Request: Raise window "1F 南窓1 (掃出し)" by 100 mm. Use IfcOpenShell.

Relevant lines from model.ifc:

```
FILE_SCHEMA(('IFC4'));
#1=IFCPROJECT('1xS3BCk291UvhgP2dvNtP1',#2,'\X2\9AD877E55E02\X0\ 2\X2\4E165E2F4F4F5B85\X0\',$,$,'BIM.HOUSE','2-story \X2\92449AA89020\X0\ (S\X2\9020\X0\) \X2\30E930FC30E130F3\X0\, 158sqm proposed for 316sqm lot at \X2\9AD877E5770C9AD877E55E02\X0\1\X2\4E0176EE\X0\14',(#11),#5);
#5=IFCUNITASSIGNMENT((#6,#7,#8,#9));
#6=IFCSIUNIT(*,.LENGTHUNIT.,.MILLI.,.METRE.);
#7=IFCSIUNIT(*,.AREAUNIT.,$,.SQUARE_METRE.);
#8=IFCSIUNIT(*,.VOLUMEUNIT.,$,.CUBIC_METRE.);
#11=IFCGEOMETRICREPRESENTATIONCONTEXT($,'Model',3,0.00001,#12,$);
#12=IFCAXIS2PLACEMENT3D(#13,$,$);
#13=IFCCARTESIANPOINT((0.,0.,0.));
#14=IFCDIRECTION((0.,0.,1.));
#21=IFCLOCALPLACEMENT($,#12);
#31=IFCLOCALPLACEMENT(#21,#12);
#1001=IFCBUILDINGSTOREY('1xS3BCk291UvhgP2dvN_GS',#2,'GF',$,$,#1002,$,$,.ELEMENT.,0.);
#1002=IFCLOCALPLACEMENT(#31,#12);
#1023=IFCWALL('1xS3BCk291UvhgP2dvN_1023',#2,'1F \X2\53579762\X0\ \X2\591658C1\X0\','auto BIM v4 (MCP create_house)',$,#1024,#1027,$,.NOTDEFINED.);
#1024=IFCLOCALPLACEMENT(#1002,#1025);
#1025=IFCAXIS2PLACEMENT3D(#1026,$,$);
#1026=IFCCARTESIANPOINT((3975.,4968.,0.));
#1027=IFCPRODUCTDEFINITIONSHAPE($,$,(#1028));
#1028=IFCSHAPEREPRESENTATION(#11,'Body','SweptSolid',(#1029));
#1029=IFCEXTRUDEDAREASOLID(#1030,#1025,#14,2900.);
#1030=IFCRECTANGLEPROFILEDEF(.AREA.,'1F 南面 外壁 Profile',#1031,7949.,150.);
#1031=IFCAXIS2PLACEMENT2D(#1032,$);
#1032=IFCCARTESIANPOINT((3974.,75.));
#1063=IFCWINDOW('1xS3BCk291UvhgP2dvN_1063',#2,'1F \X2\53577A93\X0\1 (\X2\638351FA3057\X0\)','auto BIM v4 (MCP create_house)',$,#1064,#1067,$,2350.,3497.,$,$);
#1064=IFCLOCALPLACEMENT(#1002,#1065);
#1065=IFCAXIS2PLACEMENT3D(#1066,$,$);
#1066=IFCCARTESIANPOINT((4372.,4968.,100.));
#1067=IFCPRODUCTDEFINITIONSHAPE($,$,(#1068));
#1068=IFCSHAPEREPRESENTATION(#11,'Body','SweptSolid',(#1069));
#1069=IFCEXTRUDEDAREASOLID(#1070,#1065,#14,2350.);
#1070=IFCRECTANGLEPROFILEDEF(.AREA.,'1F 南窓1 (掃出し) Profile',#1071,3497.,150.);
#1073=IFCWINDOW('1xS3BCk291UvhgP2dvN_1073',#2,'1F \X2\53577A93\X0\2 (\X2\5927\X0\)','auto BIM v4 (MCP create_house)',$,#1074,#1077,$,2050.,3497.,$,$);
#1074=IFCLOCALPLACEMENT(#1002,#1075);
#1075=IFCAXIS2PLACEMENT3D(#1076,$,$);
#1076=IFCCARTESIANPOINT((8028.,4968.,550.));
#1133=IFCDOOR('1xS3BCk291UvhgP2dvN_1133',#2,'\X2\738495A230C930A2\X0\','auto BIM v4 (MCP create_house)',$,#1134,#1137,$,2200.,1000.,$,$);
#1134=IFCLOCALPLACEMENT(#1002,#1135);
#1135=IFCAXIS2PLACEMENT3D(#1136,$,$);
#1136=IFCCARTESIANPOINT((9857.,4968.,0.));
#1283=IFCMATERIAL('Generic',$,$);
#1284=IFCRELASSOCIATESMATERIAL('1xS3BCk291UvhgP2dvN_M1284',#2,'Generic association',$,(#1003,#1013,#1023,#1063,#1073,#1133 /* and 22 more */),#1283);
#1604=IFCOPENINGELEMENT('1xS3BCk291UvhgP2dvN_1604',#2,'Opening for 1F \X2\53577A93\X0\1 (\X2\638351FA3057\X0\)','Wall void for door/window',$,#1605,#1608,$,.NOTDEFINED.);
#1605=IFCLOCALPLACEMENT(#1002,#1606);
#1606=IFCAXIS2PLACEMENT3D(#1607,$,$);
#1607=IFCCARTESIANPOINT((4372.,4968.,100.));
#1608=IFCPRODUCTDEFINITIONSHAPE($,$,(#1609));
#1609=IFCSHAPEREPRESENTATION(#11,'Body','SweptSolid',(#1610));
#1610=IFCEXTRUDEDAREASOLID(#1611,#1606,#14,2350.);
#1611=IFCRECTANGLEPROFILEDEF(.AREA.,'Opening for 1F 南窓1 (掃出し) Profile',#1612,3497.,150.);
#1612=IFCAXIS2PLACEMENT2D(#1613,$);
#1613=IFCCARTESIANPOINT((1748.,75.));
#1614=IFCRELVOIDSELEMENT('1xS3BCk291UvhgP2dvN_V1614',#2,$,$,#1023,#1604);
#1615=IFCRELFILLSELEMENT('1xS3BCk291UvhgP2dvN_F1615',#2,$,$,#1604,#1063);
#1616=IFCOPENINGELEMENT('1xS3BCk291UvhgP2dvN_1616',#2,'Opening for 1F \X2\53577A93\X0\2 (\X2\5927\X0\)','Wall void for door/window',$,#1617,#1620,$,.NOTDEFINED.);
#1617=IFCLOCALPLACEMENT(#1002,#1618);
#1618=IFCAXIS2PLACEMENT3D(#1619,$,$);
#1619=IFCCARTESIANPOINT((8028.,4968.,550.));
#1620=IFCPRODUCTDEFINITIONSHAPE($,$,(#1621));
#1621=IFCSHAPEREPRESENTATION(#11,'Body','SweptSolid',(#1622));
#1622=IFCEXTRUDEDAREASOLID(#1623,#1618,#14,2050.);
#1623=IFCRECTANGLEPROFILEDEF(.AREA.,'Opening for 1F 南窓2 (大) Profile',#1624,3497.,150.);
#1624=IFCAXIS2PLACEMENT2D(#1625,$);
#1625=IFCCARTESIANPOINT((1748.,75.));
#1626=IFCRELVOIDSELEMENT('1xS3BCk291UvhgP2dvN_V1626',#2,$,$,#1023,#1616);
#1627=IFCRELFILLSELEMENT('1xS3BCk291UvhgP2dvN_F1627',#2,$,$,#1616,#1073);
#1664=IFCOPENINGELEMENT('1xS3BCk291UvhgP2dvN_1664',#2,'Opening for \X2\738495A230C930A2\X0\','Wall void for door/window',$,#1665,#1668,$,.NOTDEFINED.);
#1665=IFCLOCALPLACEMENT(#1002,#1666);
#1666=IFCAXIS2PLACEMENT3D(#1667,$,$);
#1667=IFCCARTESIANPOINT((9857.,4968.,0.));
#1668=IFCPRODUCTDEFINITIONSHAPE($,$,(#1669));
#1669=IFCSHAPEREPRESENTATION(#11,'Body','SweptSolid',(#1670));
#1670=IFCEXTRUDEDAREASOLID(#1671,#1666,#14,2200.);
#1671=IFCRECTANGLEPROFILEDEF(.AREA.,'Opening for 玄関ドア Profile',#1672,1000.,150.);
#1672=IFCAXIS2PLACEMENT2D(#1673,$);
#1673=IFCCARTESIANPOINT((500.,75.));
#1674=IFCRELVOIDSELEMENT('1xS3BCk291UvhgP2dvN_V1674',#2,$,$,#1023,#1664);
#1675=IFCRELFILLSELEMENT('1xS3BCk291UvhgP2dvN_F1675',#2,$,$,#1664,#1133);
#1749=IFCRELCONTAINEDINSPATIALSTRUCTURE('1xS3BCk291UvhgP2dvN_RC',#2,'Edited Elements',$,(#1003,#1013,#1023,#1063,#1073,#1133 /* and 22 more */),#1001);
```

```python
import numpy as np
import ifcopenshell
import ifcopenshell.api.geometry
import ifcopenshell.util.placement
import ifcopenshell.util.unit

model = ifcopenshell.open("model.ifc")
unit_scale = ifcopenshell.util.unit.calculate_unit_scale(model)

window = model.by_guid("1xS3BCk291UvhgP2dvN_1063")
opening = window.FillsVoids[0].RelatingOpeningElement
dz = 100.0

shift = np.array([0.0, 0.0, dz])
# The window is not placed relative to its opening, so move both.
for product in (opening, window):
    matrix = ifcopenshell.util.placement.get_local_placement(product.ObjectPlacement)
    matrix[:3, 3] += shift
    ifcopenshell.api.geometry.edit_object_placement(model, product=product, matrix=matrix, is_si=False)

print(f"moved by {dz * unit_scale:+.3f} m")

model.write("model_edited.ifc")
```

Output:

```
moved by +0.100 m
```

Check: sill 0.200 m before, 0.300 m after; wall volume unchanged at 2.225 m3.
